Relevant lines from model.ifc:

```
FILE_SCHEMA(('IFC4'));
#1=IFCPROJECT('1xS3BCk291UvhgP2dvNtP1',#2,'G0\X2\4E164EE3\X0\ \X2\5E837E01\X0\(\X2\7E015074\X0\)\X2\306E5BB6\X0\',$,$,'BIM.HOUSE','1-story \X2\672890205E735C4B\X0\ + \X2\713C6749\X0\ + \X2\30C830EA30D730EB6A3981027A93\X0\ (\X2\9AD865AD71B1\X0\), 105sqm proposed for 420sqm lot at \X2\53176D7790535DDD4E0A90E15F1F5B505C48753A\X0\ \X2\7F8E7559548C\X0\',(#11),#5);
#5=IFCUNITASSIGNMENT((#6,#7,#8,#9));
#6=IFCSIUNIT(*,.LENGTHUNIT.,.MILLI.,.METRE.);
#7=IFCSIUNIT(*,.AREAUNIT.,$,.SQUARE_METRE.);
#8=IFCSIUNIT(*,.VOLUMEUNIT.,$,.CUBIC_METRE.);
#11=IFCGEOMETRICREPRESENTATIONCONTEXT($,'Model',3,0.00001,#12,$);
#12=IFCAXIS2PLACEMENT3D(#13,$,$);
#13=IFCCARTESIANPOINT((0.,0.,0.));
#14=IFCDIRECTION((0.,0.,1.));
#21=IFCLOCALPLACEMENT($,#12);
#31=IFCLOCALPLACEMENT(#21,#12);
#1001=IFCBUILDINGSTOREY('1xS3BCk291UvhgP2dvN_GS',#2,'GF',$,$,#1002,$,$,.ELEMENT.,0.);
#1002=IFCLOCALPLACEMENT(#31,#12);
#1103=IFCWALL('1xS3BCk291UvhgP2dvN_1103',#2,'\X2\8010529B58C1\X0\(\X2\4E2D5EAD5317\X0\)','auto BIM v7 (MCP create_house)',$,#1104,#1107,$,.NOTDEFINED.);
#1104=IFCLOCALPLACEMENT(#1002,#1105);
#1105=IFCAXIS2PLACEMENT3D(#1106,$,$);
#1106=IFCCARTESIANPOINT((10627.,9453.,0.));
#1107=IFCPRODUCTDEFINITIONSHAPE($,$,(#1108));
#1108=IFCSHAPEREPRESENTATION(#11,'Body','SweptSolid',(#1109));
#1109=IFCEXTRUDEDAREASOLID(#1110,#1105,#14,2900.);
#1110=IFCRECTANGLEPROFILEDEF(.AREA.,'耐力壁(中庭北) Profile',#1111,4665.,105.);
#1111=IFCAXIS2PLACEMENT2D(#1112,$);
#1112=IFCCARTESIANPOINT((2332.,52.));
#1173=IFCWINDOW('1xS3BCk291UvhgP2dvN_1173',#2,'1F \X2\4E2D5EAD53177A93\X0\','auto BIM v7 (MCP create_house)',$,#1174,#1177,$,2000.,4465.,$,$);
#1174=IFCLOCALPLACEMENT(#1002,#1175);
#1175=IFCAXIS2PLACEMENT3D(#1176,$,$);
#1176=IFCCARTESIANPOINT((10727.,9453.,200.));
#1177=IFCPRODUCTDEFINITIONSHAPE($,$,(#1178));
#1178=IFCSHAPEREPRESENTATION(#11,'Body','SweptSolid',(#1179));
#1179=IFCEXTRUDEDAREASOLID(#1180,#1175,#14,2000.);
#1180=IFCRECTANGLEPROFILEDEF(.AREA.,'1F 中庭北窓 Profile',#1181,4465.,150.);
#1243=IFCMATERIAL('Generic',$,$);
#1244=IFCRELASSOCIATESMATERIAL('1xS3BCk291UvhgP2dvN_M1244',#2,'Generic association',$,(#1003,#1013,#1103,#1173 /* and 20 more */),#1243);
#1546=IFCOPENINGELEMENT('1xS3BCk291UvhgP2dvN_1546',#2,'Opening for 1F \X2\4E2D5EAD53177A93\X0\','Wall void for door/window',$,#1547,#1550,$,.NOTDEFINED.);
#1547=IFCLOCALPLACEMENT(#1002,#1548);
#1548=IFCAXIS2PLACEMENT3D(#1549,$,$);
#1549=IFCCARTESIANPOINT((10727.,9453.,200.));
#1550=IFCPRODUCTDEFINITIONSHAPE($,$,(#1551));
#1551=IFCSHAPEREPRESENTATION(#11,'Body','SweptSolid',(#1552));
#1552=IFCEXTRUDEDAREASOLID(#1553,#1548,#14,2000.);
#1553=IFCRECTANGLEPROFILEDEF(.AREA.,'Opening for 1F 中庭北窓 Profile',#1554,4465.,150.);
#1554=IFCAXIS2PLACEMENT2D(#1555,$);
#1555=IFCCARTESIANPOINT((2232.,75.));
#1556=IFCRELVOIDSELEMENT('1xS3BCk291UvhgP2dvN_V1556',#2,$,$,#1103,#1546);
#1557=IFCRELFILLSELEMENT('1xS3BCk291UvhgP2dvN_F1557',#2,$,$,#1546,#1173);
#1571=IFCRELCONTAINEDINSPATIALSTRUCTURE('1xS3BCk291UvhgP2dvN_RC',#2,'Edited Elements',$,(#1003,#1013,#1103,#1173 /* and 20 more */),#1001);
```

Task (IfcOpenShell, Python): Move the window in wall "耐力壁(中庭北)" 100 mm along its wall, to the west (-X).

```python
import ifcopenshell
import ifcopenshell.api.geometry
import ifcopenshell.util.placement
import ifcopenshell.util.unit

model = ifcopenshell.open("model.ifc")
unit_scale = ifcopenshell.util.unit.calculate_unit_scale(model)

window = model.by_id(1173)
opening = window.FillsVoids[0].RelatingOpeningElement
wall = opening.VoidsElements[0].RelatingBuildingElement

wall_matrix = ifcopenshell.util.placement.get_local_placement(wall.ObjectPlacement)
shift = wall_matrix[:3, 0] * -0.1 / unit_scale
before = ifcopenshell.util.placement.get_local_placement(window.ObjectPlacement)[:3, 3].copy()

# The window is not placed relative to its opening, so move both.
for product in (opening, window):
    matrix = ifcopenshell.util.placement.get_local_placement(product.ObjectPlacement)
    matrix[:3, 3] += shift
    ifcopenshell.api.geometry.edit_object_placement(model, product=product, matrix=matrix, is_si=False)

after = ifcopenshell.util.placement.get_local_placement(window.ObjectPlacement)[:3, 3]
print("window moved by", (after - before).round(3) + 0.0)

model.write("model-out.ifc")
```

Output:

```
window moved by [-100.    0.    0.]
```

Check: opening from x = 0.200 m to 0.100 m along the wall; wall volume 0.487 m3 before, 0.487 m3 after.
